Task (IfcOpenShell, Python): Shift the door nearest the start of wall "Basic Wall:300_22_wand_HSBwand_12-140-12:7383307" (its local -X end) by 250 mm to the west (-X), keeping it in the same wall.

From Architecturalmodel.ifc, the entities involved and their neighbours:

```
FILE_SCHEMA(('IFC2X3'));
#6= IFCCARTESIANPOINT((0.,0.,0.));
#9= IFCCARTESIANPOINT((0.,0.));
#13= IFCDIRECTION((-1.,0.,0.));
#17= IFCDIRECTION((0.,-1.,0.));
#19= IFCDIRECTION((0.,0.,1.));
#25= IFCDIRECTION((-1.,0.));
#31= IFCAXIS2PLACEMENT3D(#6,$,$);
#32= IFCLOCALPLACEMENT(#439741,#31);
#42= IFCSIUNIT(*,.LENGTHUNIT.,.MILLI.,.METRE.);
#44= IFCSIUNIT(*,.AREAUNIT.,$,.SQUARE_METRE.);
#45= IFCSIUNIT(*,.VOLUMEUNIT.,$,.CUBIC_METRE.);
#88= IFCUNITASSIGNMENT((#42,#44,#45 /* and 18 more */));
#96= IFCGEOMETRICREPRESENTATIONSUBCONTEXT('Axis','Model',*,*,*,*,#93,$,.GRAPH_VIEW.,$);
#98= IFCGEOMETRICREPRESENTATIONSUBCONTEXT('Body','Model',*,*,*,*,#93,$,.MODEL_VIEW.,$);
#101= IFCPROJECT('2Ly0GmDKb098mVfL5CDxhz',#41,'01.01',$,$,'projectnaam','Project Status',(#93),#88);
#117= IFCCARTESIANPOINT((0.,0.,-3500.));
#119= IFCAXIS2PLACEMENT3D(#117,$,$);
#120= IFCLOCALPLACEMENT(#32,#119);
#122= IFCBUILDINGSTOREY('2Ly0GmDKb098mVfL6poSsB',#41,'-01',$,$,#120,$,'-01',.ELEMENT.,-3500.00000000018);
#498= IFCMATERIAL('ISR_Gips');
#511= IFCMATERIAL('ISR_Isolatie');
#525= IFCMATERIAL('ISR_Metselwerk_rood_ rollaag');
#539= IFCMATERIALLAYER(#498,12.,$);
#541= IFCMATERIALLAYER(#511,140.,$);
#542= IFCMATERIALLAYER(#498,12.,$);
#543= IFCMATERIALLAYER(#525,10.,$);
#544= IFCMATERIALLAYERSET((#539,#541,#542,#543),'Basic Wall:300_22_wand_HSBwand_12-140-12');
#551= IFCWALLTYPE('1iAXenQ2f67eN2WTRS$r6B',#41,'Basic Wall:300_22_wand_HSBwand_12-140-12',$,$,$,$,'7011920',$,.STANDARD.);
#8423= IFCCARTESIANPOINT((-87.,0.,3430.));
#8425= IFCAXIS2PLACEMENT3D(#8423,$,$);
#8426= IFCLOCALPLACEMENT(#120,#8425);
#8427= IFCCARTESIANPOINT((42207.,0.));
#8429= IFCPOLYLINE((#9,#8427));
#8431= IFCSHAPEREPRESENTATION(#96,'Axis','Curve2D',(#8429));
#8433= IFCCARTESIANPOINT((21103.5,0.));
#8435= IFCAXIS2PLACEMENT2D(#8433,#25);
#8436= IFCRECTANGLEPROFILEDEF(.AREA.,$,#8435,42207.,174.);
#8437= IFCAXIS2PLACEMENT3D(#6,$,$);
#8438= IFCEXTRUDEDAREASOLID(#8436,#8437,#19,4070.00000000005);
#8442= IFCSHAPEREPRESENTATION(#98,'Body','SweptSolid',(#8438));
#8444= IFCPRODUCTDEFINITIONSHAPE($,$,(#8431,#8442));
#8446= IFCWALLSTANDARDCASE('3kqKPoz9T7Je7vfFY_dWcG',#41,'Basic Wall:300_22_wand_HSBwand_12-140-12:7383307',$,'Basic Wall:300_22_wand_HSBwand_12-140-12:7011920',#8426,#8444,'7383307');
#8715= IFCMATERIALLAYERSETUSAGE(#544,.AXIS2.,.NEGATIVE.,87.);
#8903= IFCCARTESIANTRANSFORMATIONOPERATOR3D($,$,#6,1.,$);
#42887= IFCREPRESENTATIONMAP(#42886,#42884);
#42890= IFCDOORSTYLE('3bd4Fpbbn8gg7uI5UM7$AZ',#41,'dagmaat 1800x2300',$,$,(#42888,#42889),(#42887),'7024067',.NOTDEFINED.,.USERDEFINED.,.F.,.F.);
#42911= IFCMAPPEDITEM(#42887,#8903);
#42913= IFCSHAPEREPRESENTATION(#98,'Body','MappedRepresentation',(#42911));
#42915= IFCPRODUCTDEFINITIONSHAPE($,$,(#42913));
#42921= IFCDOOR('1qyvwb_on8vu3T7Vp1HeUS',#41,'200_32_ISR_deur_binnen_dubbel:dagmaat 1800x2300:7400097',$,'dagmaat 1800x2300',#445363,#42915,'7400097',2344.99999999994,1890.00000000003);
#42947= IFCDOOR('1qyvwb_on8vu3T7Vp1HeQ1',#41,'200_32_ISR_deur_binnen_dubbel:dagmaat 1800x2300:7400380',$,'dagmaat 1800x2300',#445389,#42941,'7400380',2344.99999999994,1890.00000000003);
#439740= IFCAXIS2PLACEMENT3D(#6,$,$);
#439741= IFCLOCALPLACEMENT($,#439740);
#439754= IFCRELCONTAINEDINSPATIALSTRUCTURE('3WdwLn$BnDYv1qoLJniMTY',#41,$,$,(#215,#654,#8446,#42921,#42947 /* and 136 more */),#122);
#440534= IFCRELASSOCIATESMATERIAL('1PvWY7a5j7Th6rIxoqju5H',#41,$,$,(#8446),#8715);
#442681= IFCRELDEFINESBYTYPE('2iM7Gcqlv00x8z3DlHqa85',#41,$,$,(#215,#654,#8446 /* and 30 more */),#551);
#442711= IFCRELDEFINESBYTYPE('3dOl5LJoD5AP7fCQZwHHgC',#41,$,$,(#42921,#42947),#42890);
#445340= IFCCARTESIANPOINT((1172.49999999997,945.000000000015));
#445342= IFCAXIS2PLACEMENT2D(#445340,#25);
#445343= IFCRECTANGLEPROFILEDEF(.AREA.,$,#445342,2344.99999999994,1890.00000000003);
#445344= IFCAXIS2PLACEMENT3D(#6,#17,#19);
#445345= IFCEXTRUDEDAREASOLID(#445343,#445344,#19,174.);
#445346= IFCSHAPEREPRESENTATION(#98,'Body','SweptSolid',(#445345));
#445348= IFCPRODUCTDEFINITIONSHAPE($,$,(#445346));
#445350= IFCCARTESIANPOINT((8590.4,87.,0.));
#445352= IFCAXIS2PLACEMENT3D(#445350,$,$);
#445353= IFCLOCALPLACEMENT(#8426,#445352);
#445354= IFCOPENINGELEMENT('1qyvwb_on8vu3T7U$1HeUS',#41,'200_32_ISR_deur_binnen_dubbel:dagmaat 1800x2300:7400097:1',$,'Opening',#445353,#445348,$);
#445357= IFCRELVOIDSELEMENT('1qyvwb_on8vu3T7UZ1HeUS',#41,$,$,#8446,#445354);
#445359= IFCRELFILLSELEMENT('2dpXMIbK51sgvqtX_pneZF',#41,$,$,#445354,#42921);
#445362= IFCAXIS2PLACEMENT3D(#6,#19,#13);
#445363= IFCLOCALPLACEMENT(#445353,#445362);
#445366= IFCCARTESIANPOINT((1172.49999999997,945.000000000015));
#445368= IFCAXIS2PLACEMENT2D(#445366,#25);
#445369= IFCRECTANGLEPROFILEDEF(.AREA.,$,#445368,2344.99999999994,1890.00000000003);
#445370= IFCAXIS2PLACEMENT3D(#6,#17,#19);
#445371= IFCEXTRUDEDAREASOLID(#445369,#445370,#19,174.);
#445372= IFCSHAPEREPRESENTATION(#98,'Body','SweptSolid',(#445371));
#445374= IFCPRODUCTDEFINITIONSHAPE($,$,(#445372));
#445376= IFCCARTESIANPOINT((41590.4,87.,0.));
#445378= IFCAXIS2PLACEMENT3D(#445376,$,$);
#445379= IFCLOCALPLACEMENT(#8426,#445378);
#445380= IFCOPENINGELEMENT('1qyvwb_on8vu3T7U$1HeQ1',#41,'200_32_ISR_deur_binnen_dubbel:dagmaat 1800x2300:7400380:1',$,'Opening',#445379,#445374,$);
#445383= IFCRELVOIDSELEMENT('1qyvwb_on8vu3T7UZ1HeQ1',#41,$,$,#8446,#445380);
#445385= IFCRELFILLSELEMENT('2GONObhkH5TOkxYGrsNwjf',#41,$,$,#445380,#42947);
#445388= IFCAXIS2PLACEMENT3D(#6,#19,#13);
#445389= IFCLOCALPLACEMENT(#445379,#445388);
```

```python
import ifcopenshell
import ifcopenshell.api.geometry
import ifcopenshell.util.placement

model = ifcopenshell.open("Architecturalmodel.ifc")

door = model.by_guid("1qyvwb_on8vu3T7Vp1HeUS")
opening = door.FillsVoids[0].RelatingOpeningElement
wall = opening.VoidsElements[0].RelatingBuildingElement

wall_matrix = ifcopenshell.util.placement.get_local_placement(wall.ObjectPlacement)
shift = wall_matrix[:3, 0] * -250.0
before = ifcopenshell.util.placement.get_local_placement(door.ObjectPlacement)[:3, 3].copy()

# The door is placed relative to its opening, so it follows when the opening moves.
matrix = ifcopenshell.util.placement.get_local_placement(opening.ObjectPlacement)
matrix[:3, 3] += shift
ifcopenshell.api.geometry.edit_object_placement(
    model, product=opening, matrix=matrix, is_si=False, should_transform_children=True
)

after = ifcopenshell.util.placement.get_local_placement(door.ObjectPlacement)[:3, 3]
print("door moved by", (after - before).round(3) + 0.0)

model.write("Architecturalmodel-out.ifc")
```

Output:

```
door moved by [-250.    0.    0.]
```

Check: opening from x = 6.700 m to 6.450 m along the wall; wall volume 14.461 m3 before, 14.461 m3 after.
